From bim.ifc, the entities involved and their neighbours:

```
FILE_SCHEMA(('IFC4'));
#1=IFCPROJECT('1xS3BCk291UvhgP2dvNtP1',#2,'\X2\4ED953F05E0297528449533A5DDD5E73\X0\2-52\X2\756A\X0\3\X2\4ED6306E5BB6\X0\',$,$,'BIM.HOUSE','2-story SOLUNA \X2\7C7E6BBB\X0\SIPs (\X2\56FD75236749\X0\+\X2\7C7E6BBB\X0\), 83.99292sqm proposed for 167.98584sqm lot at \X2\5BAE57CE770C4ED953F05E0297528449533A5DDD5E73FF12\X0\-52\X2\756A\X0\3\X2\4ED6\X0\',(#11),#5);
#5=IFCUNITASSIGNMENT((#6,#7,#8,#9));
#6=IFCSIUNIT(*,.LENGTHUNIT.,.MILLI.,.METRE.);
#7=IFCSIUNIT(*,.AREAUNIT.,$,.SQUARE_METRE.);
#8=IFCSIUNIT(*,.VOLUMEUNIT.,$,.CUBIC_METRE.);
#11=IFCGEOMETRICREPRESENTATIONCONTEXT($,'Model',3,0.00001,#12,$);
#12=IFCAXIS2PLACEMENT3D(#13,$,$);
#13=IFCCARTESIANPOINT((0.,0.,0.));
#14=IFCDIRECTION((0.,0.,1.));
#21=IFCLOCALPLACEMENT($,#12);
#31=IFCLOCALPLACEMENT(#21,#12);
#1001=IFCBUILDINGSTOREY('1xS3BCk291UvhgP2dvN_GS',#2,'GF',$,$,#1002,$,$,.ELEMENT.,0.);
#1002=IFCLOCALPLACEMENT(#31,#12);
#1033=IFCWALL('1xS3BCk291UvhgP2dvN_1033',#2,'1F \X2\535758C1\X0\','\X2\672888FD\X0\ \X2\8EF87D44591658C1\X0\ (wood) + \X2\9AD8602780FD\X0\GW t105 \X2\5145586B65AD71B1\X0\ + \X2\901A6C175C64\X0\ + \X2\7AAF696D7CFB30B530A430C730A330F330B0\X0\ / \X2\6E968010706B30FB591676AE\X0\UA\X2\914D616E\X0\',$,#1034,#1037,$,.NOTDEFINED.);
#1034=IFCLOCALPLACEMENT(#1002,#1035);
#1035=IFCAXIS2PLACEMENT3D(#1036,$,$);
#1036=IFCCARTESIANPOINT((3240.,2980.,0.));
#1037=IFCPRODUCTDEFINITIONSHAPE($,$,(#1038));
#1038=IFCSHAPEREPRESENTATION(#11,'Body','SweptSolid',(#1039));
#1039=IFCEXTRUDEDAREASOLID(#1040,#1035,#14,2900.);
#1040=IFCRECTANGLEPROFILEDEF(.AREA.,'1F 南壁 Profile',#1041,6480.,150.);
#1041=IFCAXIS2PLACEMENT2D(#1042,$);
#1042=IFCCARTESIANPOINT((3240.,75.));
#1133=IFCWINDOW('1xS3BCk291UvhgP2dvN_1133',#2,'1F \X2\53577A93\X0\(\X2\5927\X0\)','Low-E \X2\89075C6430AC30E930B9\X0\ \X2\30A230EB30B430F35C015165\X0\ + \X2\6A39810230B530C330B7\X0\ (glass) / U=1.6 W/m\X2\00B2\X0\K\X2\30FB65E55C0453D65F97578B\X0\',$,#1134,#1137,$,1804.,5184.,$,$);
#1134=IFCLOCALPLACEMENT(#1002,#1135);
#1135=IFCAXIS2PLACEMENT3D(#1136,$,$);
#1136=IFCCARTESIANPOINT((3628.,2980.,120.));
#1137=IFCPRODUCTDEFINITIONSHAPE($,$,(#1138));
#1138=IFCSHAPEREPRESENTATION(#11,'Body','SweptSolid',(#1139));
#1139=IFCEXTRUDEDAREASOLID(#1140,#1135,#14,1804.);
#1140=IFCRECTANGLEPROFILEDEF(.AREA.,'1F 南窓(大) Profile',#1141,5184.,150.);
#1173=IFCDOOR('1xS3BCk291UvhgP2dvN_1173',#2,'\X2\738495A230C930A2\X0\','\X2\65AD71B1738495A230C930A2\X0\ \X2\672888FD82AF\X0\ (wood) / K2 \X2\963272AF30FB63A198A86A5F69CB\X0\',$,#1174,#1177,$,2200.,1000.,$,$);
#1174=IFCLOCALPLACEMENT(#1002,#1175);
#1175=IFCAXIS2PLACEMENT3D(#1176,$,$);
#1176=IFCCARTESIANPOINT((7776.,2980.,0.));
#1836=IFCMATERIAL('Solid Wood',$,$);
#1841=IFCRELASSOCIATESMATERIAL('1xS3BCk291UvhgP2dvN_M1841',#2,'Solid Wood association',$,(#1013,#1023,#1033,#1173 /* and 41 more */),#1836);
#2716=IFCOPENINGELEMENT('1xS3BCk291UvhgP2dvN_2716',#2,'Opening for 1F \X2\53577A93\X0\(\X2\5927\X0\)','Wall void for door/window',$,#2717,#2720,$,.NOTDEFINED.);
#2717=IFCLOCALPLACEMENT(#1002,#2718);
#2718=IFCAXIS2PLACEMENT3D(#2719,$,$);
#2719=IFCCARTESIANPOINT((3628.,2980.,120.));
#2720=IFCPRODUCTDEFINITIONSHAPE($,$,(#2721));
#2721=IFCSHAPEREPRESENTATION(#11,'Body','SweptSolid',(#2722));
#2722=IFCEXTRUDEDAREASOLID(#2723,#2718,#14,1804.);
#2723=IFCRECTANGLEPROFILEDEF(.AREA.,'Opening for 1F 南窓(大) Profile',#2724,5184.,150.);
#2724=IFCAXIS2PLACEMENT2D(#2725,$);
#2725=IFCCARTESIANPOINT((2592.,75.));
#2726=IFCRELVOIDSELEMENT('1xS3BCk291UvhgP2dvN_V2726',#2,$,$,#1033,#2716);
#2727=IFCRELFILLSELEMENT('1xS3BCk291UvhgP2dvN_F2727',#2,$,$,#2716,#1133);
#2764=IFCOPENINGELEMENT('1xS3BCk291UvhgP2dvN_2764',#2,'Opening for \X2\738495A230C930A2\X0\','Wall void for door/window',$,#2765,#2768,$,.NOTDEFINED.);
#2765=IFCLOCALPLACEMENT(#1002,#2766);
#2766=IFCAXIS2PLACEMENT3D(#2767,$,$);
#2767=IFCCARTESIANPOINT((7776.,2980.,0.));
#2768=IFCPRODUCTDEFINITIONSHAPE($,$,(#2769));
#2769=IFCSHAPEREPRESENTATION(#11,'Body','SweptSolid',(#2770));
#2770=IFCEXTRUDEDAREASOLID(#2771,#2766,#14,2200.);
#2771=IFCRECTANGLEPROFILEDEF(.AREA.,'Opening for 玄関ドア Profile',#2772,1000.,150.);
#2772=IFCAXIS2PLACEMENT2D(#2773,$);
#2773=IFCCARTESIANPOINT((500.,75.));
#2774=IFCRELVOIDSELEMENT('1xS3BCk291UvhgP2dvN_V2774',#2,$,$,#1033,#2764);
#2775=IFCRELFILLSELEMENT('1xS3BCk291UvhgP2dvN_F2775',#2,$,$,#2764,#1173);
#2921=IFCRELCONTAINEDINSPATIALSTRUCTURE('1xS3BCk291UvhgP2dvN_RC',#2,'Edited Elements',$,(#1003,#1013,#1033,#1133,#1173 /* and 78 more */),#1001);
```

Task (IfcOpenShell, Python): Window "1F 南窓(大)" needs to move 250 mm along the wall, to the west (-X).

```python
import ifcopenshell
import ifcopenshell.api.geometry
import ifcopenshell.util.placement
import ifcopenshell.util.unit

model = ifcopenshell.open("bim.ifc")
unit_scale = ifcopenshell.util.unit.calculate_unit_scale(model)

window = model.by_guid("1xS3BCk291UvhgP2dvN_1133")
opening = window.FillsVoids[0].RelatingOpeningElement
wall = opening.VoidsElements[0].RelatingBuildingElement

wall_matrix = ifcopenshell.util.placement.get_local_placement(wall.ObjectPlacement)
shift = wall_matrix[:3, 0] * -0.25 / unit_scale
before = ifcopenshell.util.placement.get_local_placement(window.ObjectPlacement)[:3, 3].copy()

# The window is not placed relative to its opening, so move both.
for product in (opening, window):
    matrix = ifcopenshell.util.placement.get_local_placement(product.ObjectPlacement)
    matrix[:3, 3] += shift
    ifcopenshell.api.geometry.edit_object_placement(model, product=product, matrix=matrix, is_si=False)

after = ifcopenshell.util.placement.get_local_placement(window.ObjectPlacement)[:3, 3]
print("window moved by", (after - before).round(3) + 0.0)

model.write("bim_v2.ifc")
```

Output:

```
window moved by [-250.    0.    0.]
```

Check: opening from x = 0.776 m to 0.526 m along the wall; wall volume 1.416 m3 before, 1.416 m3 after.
